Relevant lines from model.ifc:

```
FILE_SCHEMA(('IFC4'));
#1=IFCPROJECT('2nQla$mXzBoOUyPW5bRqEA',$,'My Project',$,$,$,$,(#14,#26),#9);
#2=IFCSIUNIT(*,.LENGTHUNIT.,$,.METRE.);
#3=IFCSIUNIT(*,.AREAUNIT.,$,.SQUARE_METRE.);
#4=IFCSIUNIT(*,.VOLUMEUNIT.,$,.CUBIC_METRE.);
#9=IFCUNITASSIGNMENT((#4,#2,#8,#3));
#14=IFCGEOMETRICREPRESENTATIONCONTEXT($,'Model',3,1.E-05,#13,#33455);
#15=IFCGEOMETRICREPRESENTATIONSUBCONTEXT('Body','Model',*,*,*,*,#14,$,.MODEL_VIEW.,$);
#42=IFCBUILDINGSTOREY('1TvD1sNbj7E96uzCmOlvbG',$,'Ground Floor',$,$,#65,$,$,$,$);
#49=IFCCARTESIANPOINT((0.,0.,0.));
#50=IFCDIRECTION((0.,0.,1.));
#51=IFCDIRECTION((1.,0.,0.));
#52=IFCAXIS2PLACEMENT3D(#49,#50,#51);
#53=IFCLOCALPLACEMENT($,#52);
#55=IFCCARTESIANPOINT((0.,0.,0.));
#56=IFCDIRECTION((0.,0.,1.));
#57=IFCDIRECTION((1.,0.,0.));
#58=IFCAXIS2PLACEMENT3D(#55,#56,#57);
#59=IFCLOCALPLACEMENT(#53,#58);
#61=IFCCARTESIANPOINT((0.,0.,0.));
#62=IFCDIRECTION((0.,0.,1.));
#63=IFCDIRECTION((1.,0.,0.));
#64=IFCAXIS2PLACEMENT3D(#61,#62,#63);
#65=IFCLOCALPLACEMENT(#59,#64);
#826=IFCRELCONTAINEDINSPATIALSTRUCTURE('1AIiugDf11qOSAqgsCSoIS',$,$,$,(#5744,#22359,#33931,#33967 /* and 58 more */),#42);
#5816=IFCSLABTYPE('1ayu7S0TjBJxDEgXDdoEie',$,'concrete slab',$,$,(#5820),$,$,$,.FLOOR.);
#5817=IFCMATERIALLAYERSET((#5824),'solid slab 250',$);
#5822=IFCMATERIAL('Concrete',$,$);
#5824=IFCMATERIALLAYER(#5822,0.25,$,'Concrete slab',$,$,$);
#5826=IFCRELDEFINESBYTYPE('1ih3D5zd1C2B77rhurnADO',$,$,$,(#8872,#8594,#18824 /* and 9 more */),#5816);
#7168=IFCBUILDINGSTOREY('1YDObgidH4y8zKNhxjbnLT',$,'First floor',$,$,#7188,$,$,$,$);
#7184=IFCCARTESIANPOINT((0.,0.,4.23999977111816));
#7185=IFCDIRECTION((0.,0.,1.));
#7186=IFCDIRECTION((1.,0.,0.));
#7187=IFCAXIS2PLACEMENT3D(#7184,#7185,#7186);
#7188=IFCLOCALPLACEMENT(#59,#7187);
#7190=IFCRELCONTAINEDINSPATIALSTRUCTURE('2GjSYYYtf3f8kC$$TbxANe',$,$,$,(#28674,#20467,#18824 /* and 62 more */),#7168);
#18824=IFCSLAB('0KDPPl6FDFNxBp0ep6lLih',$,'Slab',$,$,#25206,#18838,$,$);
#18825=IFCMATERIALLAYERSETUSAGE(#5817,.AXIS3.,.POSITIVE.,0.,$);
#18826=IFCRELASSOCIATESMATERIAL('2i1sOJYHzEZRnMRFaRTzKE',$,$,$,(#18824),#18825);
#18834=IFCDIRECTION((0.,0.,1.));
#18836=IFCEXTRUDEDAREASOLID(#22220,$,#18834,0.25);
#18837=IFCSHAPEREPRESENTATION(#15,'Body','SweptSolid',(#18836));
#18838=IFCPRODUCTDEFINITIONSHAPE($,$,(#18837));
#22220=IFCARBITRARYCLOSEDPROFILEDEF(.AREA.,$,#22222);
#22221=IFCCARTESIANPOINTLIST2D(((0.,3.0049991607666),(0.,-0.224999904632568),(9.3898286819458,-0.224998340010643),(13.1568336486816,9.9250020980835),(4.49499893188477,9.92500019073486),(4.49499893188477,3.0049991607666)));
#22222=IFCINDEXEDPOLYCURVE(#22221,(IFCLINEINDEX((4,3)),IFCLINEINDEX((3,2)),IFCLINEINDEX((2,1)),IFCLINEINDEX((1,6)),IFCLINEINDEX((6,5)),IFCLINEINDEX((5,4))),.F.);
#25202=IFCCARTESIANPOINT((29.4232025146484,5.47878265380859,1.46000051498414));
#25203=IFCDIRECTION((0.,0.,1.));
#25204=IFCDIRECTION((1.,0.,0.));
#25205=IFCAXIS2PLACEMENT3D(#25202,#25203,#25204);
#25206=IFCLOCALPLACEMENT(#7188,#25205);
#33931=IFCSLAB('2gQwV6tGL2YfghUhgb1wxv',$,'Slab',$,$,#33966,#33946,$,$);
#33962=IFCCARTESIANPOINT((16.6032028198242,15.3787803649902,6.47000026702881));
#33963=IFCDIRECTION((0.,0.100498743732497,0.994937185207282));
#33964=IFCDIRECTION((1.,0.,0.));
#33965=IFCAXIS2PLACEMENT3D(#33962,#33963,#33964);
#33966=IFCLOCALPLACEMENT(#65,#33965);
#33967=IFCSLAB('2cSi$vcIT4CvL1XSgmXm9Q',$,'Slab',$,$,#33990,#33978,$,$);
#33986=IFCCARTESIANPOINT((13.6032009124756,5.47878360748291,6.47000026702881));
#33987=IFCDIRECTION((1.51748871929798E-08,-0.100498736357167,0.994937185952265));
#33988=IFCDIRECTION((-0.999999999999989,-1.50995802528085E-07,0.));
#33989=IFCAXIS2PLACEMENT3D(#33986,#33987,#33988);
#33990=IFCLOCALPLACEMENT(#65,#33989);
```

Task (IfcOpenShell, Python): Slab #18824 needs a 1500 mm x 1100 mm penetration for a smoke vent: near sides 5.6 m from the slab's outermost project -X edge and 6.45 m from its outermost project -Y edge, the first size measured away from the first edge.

```python
import numpy as np
import ifcopenshell
import ifcopenshell.api.feature
import ifcopenshell.api.geometry
import ifcopenshell.api.root
import ifcopenshell.geom
import ifcopenshell.util.placement
import ifcopenshell.util.representation
import ifcopenshell.util.shape
import ifcopenshell.util.unit

model = ifcopenshell.open("model.ifc")
unit_scale = ifcopenshell.util.unit.calculate_unit_scale(model)
settings = ifcopenshell.geom.settings()


def volume(element):
    """Net volume in cubic metres, openings subtracted."""
    shape = ifcopenshell.geom.create_shape(settings, element)
    return ifcopenshell.util.shape.get_volume(shape.geometry)


slab = model.by_id(18824)
before = volume(slab)

# Extent in the slab's own axes, in metres. The edges named are its -X and -Y sides.
slab_shape = ifcopenshell.geom.create_shape(settings, slab)
vertices = ifcopenshell.util.shape.get_vertices(slab_shape.geometry)
x_min, y_min, bottom = vertices.min(axis=0)
top = vertices[:, 2].max()

opening = ifcopenshell.api.root.create_entity(model, ifc_class="IfcOpeningElement", name="Smoke vent opening", predefined_type="OPENING")
context = ifcopenshell.util.representation.get_context(model, "Model", "Body", "MODEL_VIEW")
width, depth = 1.5, 1.1
outline = [(0.0, 0.0), (width, 0.0), (width, depth), (0.0, depth), (0.0, 0.0)]
# Overshoot both faces by 50 mm so the cut is clean.
shape = ifcopenshell.api.geometry.add_slab_representation(
    model, context=context, depth=top - bottom + 0.1, polyline=outline
)
ifcopenshell.api.geometry.assign_representation(model, product=opening, representation=shape)

matrix = ifcopenshell.util.placement.get_local_placement(slab.ObjectPlacement)
matrix[:, 3] = matrix @ np.append(np.array([x_min + 5.6, y_min + 6.45, bottom - 0.05]) / unit_scale, 1.0)
ifcopenshell.api.geometry.edit_object_placement(model, product=opening, matrix=matrix, is_si=False)
ifcopenshell.api.feature.add_feature(model, feature=opening, element=slab)

after = volume(slab)

print(f"slab volume {before:.3f} -> {after:.3f} m3")

model.write("model_v2.ifc")
```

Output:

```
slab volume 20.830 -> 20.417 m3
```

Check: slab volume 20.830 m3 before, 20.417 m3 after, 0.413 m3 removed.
